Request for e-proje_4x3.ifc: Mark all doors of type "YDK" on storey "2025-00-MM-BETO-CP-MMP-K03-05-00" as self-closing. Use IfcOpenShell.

First a look at what the model holds.

```python
import ifcopenshell
import ifcopenshell.util.element

model = ifcopenshell.open("e-proje_4x3.ifc")
print(model.schema)
storey = next(s for s in model.by_type("IfcBuildingStorey") if s.Name == "2025-00-MM-BETO-CP-MMP-K03-05-00")
doors = [e for e in ifcopenshell.util.element.get_decomposition(storey) if e.is_a("IfcDoor")]
seen = {}
for e in doors:
    element_type = ifcopenshell.util.element.get_type(e)
    key = (element_type.Name if element_type != e and element_type else None, ifcopenshell.util.element.get_pset(e, "Pset_DoorCommon", "SelfClosing"))
    seen[key] = seen.get(key, 0) + 1
for (name, value), count in sorted(seen.items(), key=str):
    print(count, "x", name, "|", value)
```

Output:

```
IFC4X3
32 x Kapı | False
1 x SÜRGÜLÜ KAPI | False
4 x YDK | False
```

```python
import ifcopenshell
import ifcopenshell.api.pset
import ifcopenshell.util.element

model = ifcopenshell.open("e-proje_4x3.ifc")

storey = next(s for s in model.by_type("IfcBuildingStorey") if s.Name == "2025-00-MM-BETO-CP-MMP-K03-05-00")
doors = [e for e in ifcopenshell.util.element.get_decomposition(storey) if e.is_a("IfcDoor")]

count = 0
for e in doors:
    element_type = ifcopenshell.util.element.get_type(e)
    if element_type in (None, e) or element_type.Name != "YDK":
        continue
    # add_pset returns the element's existing set when there is one.
    pset = ifcopenshell.api.pset.add_pset(model, product=e, name="Pset_DoorCommon")
    ifcopenshell.api.pset.edit_pset(model, pset=pset, properties={"SelfClosing": True})
    count += 1

print(count, "doors updated")

model.write("e-proje_4x3_rev.ifc")
```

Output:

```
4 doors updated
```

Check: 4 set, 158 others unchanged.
